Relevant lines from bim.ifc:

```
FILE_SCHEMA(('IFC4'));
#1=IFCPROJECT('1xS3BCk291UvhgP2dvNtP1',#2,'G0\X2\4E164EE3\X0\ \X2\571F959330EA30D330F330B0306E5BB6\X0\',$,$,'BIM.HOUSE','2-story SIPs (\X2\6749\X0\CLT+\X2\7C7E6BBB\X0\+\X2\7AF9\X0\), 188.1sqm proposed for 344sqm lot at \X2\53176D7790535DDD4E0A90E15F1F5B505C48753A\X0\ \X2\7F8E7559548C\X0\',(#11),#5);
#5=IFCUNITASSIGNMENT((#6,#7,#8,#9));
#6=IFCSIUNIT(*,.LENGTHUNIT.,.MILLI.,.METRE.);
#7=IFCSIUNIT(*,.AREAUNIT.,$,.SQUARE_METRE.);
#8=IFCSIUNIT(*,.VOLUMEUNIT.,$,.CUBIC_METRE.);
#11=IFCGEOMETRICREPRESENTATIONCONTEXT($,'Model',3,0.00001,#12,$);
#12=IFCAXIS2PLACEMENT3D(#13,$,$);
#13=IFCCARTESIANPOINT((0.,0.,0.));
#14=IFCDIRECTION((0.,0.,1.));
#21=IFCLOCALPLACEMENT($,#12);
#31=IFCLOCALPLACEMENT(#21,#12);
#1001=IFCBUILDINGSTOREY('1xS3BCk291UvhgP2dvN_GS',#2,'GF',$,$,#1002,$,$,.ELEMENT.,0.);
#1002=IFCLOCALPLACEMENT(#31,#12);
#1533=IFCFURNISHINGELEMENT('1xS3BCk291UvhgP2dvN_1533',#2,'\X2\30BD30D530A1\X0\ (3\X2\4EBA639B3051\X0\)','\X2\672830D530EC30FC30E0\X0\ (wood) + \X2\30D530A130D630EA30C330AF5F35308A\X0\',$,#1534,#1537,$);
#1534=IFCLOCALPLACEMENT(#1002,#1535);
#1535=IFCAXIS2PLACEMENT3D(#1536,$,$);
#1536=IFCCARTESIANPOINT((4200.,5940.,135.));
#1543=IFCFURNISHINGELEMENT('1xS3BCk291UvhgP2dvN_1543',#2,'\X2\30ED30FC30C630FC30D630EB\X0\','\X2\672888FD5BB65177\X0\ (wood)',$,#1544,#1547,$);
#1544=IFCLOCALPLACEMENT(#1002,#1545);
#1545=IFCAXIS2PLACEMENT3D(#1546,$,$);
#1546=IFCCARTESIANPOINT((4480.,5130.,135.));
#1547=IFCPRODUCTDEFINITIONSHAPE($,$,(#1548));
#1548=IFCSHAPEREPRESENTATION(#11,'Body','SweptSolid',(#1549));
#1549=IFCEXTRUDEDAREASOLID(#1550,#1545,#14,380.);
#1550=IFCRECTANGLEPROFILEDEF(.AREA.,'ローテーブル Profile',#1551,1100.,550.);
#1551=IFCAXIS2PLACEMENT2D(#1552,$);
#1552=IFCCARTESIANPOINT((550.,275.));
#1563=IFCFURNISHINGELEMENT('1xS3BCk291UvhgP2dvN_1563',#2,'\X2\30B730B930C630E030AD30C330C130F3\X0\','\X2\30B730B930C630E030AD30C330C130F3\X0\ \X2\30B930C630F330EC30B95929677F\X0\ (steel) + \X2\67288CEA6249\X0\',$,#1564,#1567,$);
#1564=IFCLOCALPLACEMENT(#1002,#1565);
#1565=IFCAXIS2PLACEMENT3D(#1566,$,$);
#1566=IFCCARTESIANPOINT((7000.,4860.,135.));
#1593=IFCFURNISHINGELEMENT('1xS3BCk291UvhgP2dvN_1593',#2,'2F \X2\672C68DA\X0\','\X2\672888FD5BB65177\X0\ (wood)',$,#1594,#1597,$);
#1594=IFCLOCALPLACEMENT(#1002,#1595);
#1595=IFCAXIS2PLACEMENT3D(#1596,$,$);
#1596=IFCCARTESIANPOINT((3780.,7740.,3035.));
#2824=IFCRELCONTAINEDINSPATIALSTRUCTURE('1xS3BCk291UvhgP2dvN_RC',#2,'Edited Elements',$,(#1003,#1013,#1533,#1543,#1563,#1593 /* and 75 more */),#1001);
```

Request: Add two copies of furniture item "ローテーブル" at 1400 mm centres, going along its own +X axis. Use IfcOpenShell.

```python
import ifcopenshell
import ifcopenshell.api.geometry
import ifcopenshell.api.root
import ifcopenshell.util.element
import ifcopenshell.util.placement

model = ifcopenshell.open("bim.ifc")


def reuse_history(source, copy):
    """copy_class also copies each property set's owner history, people and application; keep the originals."""
    for rel in copy.IsDefinedBy:
        if rel.is_a("IfcRelDefinesByProperties") and (history := rel.RelatingPropertyDefinition.OwnerHistory):
            rel.RelatingPropertyDefinition.OwnerHistory = source.OwnerHistory
            ifcopenshell.util.element.remove_deep2(model, history)


source = model.by_id(1543)
base = ifcopenshell.util.placement.get_local_placement(source.ObjectPlacement)
step = base[:3, 0] * 1400.0

for i in range(1, 3):
    copy = ifcopenshell.api.root.copy_class(model, product=source)
    copy.Representation = ifcopenshell.util.element.copy_deep(
        model, source.Representation, exclude=["IfcGeometricRepresentationContext", "IfcRepresentationMap"]
    )
    reuse_history(source, copy)
    matrix = base.copy()
    matrix[:3, 3] += i * step
    print("added at", matrix[:3, 3].round(3) + 0.0)
    ifcopenshell.api.geometry.edit_object_placement(model, product=copy, matrix=matrix, is_si=False)

model.write("bim-out.ifc")
```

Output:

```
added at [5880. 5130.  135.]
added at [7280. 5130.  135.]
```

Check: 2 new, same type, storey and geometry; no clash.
